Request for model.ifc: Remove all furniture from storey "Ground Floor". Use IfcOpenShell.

First a look at what the model holds.

```python
import ifcopenshell
import ifcopenshell.util.element

model = ifcopenshell.open("model.ifc")
print(model.schema)
storey = next(s for s in model.by_type("IfcBuildingStorey") if s.Name == "Ground Floor")
furniture = [e for e in ifcopenshell.util.element.get_decomposition(storey) if e.is_a("IfcFurnishingElement")]
seen = {}
for e in furniture:
    element_type = ifcopenshell.util.element.get_type(e)
    name = element_type.Name if element_type not in (None, e) else None
    seen[name] = seen.get(name, 0) + 1
for name, count in sorted(seen.items(), key=str):
    print(count, "x", name)
```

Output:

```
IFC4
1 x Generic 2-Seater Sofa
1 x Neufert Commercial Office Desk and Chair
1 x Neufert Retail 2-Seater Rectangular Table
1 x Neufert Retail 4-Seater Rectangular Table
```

```python
import ifcopenshell
import ifcopenshell.api.root
import ifcopenshell.util.element

model = ifcopenshell.open("model.ifc")

storey = next(s for s in model.by_type("IfcBuildingStorey") if s.Name == "Ground Floor")
furniture = [e for e in ifcopenshell.util.element.get_decomposition(storey) if e.is_a("IfcFurnishingElement")]

for e in furniture:
    ifcopenshell.api.root.remove_product(model, product=e)
print(len(furniture), "removed")

model.write("model_edited.ifc")
```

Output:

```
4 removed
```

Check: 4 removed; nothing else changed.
